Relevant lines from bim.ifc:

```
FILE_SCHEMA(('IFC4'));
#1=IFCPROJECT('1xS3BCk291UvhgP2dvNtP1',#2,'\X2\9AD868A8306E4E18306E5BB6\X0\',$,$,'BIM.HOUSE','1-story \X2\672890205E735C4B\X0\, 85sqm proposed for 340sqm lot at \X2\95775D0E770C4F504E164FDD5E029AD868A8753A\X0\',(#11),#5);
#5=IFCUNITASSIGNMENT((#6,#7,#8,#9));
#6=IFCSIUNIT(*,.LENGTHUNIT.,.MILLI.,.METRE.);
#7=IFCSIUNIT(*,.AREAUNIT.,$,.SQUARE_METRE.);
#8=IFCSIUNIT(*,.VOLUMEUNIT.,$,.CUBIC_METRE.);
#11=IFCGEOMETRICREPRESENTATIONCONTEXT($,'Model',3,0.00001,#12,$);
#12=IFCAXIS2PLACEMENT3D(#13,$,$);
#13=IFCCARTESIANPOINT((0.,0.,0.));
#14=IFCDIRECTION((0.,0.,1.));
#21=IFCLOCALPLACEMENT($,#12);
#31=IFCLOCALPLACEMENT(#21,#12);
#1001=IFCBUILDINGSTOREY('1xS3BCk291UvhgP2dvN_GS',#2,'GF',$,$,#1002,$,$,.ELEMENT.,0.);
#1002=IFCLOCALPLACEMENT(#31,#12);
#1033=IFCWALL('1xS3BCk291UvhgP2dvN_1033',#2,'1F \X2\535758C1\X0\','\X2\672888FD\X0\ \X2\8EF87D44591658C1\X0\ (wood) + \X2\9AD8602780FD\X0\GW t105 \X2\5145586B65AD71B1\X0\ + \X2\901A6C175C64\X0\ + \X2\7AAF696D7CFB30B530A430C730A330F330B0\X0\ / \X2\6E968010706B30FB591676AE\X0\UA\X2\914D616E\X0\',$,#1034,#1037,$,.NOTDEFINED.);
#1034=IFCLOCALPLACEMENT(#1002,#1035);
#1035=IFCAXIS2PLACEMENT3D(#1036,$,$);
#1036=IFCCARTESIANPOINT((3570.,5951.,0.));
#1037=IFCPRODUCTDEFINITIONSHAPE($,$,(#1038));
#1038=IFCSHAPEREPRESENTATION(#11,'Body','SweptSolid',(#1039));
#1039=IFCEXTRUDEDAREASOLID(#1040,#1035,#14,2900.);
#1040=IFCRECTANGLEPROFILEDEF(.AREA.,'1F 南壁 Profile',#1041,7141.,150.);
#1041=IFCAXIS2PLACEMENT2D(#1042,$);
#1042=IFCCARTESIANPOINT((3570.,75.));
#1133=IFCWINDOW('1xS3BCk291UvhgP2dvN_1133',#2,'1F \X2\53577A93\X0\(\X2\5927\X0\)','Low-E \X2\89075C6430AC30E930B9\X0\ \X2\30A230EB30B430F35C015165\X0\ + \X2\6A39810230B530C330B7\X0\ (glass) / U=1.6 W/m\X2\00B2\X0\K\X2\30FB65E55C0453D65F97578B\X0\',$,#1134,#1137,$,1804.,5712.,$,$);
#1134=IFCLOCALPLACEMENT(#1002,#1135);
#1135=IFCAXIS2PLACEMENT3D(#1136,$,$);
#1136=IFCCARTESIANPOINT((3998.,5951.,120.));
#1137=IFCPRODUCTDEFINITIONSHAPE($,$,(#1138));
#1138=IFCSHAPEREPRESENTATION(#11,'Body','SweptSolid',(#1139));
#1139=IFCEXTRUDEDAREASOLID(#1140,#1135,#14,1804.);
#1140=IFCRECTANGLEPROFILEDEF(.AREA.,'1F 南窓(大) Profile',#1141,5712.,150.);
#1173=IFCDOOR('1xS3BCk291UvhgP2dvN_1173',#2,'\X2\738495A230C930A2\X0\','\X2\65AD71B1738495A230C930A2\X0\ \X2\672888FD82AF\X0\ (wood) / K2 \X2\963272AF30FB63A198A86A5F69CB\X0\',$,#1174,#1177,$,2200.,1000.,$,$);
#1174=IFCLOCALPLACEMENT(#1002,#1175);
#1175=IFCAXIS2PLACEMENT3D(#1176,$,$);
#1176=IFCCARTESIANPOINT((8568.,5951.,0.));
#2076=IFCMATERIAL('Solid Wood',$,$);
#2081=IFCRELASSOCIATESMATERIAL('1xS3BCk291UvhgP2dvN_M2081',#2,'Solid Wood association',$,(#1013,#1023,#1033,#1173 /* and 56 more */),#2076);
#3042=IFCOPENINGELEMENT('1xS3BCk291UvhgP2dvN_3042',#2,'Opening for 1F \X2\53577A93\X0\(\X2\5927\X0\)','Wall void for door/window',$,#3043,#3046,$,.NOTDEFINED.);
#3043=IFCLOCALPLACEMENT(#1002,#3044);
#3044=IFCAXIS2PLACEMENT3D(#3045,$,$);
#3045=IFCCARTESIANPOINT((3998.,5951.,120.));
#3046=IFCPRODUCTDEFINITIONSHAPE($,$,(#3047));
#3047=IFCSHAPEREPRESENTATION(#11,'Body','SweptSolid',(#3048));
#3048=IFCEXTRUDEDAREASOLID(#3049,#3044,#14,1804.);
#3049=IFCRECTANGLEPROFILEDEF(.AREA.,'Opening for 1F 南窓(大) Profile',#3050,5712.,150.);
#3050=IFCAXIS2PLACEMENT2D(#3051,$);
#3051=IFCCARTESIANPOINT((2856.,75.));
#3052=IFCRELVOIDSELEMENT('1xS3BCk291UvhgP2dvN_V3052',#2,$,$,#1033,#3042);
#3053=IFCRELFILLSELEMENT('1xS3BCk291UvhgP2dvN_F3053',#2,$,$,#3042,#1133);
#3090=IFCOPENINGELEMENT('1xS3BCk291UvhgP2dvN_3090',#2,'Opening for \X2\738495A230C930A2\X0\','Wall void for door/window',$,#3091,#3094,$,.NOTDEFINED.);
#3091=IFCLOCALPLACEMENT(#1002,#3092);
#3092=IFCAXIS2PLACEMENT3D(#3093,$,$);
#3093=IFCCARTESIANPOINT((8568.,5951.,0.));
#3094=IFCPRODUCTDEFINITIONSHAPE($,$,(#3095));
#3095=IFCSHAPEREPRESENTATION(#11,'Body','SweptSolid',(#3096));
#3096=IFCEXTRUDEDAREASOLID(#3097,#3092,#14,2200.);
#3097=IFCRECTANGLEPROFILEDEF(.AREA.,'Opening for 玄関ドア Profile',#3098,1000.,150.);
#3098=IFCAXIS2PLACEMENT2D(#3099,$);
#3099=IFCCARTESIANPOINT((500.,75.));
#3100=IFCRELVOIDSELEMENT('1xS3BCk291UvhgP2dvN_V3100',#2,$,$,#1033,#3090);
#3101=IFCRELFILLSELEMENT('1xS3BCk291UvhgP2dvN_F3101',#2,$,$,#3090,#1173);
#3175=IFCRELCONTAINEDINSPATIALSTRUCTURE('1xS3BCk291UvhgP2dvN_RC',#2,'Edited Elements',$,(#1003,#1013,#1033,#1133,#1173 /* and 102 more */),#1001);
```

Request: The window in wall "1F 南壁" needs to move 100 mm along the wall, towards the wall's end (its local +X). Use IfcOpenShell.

```python
import ifcopenshell
import ifcopenshell.api.geometry
import ifcopenshell.util.placement

model = ifcopenshell.open("bim.ifc")

window = model.by_guid("1xS3BCk291UvhgP2dvN_1133")
opening = window.FillsVoids[0].RelatingOpeningElement
wall = opening.VoidsElements[0].RelatingBuildingElement

wall_matrix = ifcopenshell.util.placement.get_local_placement(wall.ObjectPlacement)
shift = wall_matrix[:3, 0] * 100.0
before = ifcopenshell.util.placement.get_local_placement(window.ObjectPlacement)[:3, 3].copy()

# The window is not placed relative to its opening, so move both.
for product in (opening, window):
    matrix = ifcopenshell.util.placement.get_local_placement(product.ObjectPlacement)
    matrix[:3, 3] += shift
    ifcopenshell.api.geometry.edit_object_placement(model, product=product, matrix=matrix, is_si=False)

after = ifcopenshell.util.placement.get_local_placement(window.ObjectPlacement)[:3, 3]
print("window moved by", (after - before).round(3) + 0.0)

model.write("bim_v2.ifc")
```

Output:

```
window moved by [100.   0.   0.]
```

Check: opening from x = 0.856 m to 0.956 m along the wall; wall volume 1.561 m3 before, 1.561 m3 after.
